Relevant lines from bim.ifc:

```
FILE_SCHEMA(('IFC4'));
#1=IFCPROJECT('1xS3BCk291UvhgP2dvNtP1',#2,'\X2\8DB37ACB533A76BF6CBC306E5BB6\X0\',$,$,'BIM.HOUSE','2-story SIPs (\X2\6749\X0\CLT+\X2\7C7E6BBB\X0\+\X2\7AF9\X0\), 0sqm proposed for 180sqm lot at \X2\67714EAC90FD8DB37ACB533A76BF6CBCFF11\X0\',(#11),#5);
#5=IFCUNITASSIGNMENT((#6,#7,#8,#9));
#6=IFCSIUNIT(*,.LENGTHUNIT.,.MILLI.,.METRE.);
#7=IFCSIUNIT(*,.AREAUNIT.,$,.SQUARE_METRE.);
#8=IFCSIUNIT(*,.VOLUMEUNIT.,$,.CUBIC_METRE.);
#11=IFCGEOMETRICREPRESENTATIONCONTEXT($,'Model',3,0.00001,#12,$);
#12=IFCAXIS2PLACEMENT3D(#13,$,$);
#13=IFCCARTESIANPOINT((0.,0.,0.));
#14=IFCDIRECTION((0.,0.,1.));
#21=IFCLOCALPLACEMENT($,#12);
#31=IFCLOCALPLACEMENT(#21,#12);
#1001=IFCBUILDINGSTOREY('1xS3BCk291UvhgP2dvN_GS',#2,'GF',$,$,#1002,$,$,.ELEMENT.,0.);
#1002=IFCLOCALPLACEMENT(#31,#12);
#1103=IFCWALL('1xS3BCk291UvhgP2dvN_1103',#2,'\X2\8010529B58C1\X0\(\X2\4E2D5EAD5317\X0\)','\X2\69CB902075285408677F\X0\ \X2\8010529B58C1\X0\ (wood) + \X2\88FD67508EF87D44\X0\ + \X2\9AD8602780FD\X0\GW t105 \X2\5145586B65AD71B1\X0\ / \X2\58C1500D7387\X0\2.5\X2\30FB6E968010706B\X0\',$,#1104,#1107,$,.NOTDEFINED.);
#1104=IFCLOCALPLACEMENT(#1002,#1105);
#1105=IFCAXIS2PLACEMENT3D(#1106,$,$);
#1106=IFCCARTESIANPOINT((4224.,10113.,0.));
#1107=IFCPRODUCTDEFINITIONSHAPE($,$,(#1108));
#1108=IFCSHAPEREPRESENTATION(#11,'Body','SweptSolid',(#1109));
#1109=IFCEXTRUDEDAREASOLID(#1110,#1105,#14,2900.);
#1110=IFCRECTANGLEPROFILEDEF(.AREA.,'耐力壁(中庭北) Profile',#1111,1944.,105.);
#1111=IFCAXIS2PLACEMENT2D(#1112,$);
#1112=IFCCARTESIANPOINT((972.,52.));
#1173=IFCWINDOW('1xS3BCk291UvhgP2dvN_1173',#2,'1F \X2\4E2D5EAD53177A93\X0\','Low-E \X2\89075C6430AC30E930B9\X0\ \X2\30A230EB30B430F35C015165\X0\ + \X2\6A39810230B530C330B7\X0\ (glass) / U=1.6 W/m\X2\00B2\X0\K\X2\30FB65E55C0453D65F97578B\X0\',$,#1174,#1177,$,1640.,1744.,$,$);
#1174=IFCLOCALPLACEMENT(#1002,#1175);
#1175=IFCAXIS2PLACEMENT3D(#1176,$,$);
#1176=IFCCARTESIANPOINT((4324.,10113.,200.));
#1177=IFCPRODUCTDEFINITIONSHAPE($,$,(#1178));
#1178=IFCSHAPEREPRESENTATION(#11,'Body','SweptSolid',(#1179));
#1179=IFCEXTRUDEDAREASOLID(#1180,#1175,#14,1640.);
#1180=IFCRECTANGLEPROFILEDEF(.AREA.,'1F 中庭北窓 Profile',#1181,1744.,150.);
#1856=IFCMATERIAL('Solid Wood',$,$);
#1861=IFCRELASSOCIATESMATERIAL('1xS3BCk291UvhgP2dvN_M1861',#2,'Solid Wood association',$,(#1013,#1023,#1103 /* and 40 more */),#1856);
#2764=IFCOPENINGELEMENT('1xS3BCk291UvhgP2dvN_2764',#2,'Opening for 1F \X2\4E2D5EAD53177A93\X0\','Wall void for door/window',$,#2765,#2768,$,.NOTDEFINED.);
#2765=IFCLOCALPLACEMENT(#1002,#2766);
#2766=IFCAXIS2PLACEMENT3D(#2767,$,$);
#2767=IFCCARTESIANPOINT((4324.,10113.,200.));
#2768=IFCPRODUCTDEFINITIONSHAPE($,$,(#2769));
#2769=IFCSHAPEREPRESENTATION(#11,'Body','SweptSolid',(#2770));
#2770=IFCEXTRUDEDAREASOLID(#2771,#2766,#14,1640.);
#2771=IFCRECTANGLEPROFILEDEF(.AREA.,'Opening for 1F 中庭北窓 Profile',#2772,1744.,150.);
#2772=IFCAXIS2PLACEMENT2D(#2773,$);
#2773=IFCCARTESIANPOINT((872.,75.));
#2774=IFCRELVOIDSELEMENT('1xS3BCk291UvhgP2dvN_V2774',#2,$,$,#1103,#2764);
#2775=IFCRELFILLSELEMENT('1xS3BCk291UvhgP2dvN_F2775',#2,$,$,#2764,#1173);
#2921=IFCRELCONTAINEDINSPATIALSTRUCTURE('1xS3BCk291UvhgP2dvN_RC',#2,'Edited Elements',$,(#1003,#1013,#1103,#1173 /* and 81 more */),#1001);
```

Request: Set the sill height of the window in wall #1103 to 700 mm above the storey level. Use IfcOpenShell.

```python
import numpy as np
import ifcopenshell
import ifcopenshell.api.geometry
import ifcopenshell.geom
import ifcopenshell.util.element
import ifcopenshell.util.placement
import ifcopenshell.util.shape
import ifcopenshell.util.unit

model = ifcopenshell.open("bim.ifc")
unit_scale = ifcopenshell.util.unit.calculate_unit_scale(model)

window = model.by_guid("1xS3BCk291UvhgP2dvN_1173")
opening = window.FillsVoids[0].RelatingOpeningElement
storey = ifcopenshell.util.element.get_container(window, ifc_class="IfcBuildingStorey")
level = ifcopenshell.util.placement.get_local_placement(storey.ObjectPlacement)[2, 3]

# The opening's origin need not be at the sill, so measure its lowest point.
shape = ifcopenshell.geom.create_shape(ifcopenshell.geom.settings(), opening)
bottom = ifcopenshell.util.shape.get_shape_bottom_elevation(shape, shape.geometry) / unit_scale
dz = level + 700.0 - bottom

shift = np.array([0.0, 0.0, dz])
# The window is not placed relative to its opening, so move both.
for product in (opening, window):
    matrix = ifcopenshell.util.placement.get_local_placement(product.ObjectPlacement)
    matrix[:3, 3] += shift
    ifcopenshell.api.geometry.edit_object_placement(model, product=product, matrix=matrix, is_si=False)

print(f"moved by {dz * unit_scale:+.3f} m")

model.write("bim_updated.ifc")
```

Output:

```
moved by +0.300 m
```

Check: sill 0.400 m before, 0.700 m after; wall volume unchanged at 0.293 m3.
